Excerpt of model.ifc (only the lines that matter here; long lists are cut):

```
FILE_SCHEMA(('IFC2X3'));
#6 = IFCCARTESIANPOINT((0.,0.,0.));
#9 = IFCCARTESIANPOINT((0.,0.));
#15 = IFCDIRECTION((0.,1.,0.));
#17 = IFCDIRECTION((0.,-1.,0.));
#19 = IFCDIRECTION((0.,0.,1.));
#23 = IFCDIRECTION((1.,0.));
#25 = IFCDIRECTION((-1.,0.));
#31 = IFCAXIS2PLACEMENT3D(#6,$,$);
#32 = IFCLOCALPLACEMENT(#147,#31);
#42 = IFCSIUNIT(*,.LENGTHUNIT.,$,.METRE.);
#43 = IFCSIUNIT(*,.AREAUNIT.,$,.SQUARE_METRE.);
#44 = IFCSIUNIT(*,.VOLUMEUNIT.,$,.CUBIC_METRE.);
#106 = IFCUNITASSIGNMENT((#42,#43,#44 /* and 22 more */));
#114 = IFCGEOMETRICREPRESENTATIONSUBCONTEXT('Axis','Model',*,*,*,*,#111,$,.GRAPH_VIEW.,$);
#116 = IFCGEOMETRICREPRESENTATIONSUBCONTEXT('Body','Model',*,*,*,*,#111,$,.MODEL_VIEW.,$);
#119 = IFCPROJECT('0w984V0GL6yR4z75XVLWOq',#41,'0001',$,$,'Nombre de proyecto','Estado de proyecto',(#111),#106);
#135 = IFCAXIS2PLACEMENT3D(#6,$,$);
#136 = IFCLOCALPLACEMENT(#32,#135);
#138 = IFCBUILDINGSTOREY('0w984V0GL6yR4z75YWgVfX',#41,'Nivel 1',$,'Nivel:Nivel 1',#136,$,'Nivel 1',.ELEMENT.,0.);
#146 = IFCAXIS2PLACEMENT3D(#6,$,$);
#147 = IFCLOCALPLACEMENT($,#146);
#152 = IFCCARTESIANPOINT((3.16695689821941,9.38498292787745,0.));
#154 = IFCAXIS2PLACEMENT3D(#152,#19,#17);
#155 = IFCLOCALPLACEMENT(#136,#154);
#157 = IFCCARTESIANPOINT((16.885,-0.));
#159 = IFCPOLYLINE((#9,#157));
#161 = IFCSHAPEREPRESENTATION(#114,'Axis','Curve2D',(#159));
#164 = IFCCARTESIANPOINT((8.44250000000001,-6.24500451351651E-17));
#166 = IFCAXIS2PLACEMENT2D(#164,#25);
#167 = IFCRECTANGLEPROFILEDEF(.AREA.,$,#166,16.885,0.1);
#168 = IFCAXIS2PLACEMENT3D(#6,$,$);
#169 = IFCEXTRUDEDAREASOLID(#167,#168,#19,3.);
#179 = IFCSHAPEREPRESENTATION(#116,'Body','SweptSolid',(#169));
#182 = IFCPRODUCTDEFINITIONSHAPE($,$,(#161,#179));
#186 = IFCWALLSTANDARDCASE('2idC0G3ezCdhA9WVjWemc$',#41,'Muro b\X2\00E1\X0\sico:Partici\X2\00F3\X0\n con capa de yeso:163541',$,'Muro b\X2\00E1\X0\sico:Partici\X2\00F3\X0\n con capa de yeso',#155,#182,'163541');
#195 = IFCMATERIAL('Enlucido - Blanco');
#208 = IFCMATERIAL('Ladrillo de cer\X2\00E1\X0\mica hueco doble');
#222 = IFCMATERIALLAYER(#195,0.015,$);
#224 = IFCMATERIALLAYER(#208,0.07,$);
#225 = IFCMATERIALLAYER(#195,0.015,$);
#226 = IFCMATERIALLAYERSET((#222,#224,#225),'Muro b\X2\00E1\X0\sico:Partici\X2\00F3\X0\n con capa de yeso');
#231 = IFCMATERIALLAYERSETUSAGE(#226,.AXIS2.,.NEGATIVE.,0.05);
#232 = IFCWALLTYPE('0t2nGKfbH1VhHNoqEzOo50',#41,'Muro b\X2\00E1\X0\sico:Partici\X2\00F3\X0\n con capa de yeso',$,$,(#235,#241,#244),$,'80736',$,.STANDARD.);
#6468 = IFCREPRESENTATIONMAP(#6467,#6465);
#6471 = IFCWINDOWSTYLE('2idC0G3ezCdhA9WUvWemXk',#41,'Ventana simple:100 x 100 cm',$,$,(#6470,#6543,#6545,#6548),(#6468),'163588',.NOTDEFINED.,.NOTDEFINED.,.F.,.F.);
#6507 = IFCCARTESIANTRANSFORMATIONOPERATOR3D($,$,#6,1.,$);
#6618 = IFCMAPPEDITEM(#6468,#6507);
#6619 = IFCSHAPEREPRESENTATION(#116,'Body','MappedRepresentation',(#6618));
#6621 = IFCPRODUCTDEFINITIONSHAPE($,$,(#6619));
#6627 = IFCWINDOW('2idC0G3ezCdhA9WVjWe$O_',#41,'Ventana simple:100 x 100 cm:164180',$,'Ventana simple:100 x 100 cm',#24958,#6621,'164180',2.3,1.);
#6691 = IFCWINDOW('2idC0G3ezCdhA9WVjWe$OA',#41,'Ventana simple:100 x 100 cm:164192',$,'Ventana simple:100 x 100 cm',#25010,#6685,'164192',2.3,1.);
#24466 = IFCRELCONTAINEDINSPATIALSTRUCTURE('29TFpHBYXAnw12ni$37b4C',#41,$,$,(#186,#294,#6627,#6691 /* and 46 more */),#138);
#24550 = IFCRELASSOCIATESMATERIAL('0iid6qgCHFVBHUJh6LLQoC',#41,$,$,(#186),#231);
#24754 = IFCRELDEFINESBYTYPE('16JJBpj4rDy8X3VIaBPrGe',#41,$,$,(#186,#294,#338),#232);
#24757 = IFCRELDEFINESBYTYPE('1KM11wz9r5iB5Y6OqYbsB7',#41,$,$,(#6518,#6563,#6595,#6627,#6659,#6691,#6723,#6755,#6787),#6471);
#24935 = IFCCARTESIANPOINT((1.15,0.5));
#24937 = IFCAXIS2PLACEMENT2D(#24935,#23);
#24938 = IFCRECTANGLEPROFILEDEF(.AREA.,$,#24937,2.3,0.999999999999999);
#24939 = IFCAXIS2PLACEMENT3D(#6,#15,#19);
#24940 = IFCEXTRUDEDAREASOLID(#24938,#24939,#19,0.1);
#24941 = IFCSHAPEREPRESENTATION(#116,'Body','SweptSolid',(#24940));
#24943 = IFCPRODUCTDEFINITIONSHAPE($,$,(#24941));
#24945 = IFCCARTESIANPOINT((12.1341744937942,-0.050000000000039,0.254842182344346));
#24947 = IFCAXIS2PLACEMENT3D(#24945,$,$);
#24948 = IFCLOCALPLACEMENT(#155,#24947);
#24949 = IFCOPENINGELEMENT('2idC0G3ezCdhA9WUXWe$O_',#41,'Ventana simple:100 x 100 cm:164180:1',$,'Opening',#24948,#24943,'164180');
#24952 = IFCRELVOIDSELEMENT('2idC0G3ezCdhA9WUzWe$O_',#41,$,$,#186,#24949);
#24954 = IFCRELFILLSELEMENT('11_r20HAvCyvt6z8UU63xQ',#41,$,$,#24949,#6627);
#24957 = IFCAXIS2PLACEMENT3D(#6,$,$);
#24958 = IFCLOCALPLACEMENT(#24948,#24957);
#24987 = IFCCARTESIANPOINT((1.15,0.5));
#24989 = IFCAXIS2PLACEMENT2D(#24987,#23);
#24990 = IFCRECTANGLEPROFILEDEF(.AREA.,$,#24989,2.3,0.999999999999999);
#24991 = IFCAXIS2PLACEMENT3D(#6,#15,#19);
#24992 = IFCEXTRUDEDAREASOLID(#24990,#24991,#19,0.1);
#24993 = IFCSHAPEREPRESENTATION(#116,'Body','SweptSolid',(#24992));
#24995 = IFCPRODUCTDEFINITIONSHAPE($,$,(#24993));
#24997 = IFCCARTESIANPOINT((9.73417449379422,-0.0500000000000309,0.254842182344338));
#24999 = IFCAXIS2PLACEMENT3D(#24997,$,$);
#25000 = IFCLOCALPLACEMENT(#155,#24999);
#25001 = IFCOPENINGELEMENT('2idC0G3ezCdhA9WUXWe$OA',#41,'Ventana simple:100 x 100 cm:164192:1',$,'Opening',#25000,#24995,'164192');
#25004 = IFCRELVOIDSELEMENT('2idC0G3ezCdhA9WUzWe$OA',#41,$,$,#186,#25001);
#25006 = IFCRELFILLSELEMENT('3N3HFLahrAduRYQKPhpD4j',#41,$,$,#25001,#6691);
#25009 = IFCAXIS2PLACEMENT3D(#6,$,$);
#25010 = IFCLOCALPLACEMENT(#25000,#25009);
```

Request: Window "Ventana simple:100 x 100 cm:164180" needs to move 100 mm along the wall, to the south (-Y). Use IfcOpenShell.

```python
import ifcopenshell
import ifcopenshell.api.geometry
import ifcopenshell.util.placement
import ifcopenshell.util.unit

model = ifcopenshell.open("model.ifc")
unit_scale = ifcopenshell.util.unit.calculate_unit_scale(model)

window = model.by_guid("2idC0G3ezCdhA9WVjWe$O_")
opening = window.FillsVoids[0].RelatingOpeningElement
wall = opening.VoidsElements[0].RelatingBuildingElement

wall_matrix = ifcopenshell.util.placement.get_local_placement(wall.ObjectPlacement)
shift = wall_matrix[:3, 0] * 0.1 / unit_scale
before = ifcopenshell.util.placement.get_local_placement(window.ObjectPlacement)[:3, 3].copy()

# The window is placed relative to its opening, so it follows when the opening moves.
matrix = ifcopenshell.util.placement.get_local_placement(opening.ObjectPlacement)
matrix[:3, 3] += shift
ifcopenshell.api.geometry.edit_object_placement(
    model, product=opening, matrix=matrix, is_si=False, should_transform_children=True
)

after = ifcopenshell.util.placement.get_local_placement(window.ObjectPlacement)[:3, 3]
print("window moved by", (after - before).round(3) + 0.0)

model.write("model_rev.ifc")
```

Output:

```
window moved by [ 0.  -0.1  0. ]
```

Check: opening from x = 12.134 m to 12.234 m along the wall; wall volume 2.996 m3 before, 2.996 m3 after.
